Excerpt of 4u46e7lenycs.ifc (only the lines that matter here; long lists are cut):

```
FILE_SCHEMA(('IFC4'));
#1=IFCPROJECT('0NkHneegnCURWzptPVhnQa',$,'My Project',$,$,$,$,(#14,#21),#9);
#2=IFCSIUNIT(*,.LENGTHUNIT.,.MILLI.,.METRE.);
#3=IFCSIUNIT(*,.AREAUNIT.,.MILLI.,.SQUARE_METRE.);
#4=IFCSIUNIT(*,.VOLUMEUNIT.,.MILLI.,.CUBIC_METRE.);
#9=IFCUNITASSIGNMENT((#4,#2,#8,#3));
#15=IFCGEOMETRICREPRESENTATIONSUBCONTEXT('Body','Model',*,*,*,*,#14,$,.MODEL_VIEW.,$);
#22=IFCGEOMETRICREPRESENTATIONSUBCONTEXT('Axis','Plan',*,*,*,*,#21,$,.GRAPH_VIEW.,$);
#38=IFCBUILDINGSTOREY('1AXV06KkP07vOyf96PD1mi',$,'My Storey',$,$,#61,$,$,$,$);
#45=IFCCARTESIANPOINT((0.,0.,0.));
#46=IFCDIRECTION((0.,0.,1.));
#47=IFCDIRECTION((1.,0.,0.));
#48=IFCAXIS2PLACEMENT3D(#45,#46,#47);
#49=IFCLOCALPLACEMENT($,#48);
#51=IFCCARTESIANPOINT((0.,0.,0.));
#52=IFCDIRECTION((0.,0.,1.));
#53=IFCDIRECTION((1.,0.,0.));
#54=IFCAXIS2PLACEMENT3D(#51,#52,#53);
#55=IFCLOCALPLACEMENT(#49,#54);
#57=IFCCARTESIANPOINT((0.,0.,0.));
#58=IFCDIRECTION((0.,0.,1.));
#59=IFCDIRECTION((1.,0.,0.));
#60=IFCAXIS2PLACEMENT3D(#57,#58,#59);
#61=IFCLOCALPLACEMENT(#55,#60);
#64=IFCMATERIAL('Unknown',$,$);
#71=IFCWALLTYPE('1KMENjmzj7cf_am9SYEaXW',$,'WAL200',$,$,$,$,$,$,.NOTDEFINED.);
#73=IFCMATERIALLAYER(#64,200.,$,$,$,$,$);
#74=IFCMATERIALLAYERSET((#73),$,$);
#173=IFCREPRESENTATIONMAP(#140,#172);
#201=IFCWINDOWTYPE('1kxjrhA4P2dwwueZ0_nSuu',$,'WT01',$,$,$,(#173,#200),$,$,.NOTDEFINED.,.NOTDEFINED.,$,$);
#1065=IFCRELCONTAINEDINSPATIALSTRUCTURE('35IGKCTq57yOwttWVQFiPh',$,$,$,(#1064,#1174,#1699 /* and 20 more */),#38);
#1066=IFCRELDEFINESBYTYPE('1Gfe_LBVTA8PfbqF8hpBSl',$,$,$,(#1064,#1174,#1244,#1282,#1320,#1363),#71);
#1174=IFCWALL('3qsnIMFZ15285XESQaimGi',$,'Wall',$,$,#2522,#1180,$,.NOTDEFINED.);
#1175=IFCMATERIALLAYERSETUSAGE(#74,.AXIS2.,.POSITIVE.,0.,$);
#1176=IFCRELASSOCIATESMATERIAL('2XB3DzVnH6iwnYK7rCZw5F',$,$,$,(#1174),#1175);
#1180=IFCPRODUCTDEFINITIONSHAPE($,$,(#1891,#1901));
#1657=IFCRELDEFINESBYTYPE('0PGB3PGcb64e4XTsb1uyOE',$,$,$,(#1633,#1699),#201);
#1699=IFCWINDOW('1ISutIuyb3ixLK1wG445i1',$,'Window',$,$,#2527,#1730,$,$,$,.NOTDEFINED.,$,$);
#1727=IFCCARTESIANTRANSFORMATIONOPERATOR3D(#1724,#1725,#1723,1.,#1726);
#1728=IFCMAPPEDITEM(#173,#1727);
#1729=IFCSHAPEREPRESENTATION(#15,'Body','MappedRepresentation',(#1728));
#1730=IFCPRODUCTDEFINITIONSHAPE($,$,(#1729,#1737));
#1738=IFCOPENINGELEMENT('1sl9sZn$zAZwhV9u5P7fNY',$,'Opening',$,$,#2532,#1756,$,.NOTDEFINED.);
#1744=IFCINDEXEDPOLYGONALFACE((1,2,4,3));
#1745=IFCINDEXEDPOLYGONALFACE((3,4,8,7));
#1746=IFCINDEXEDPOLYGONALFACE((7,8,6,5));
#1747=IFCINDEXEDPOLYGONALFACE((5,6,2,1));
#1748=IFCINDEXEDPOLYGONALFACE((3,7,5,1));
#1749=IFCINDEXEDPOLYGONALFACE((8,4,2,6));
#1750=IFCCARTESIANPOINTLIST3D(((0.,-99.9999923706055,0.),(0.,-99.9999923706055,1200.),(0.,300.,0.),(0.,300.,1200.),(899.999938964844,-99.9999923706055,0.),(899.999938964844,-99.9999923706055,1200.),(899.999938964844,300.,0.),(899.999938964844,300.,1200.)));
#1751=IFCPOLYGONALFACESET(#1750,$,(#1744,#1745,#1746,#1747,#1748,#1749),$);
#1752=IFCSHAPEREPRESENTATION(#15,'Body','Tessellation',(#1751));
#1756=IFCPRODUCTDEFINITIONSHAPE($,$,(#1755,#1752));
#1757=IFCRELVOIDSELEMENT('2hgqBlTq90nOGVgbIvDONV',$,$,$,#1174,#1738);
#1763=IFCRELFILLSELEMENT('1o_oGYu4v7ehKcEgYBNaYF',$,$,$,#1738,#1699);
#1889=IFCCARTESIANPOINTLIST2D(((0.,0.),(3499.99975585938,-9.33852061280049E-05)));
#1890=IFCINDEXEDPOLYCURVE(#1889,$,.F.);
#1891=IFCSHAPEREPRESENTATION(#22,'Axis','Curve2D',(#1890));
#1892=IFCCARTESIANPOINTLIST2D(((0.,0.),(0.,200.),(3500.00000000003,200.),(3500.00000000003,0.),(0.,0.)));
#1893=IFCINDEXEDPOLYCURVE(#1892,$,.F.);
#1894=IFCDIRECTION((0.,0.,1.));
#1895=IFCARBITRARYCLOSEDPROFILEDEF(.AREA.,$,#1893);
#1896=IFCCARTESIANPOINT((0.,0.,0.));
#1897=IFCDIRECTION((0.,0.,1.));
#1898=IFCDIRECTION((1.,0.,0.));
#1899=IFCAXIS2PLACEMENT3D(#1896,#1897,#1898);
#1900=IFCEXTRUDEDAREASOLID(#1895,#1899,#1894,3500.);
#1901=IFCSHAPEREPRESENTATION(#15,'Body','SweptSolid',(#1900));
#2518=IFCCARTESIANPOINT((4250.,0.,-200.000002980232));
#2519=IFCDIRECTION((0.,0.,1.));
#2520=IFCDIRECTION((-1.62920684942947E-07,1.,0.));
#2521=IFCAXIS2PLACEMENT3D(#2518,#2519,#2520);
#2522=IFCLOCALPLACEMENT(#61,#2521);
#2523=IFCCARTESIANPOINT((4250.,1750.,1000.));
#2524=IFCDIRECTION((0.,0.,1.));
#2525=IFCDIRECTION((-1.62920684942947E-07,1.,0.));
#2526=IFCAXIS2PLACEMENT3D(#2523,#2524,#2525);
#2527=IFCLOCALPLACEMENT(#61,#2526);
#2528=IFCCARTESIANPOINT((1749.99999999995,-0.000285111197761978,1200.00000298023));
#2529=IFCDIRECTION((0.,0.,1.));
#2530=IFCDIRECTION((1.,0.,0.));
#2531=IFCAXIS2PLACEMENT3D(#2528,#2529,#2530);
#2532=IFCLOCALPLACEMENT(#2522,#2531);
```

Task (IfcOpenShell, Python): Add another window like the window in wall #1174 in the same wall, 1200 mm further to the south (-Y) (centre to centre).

```python
import ifcopenshell
import ifcopenshell.api.feature
import ifcopenshell.api.geometry
import ifcopenshell.api.root
import ifcopenshell.geom
import ifcopenshell.util.element
import ifcopenshell.util.placement
import ifcopenshell.util.shape
import ifcopenshell.util.unit

model = ifcopenshell.open("4u46e7lenycs.ifc")
unit_scale = ifcopenshell.util.unit.calculate_unit_scale(model)
settings = ifcopenshell.geom.settings()


def volume(element):
    """Net volume in cubic metres, openings subtracted."""
    shape = ifcopenshell.geom.create_shape(settings, element)
    return ifcopenshell.util.shape.get_volume(shape.geometry)


window = model.by_guid("1ISutIuyb3ixLK1wG445i1")
opening = window.FillsVoids[0].RelatingOpeningElement
wall = opening.VoidsElements[0].RelatingBuildingElement
before = volume(wall)
shift = ifcopenshell.util.placement.get_local_placement(wall.ObjectPlacement)[:3, 0] * -1.2 / unit_scale

# copy_class copies the void relationship, type, container and properties, but no geometry.
new_opening = ifcopenshell.api.root.copy_class(model, product=opening)
new_opening.Representation = ifcopenshell.util.element.copy_deep(
    model, opening.Representation, exclude=["IfcGeometricRepresentationContext", "IfcRepresentationMap"]
)
new_window = ifcopenshell.api.root.copy_class(model, product=window)
new_window.Representation = ifcopenshell.util.element.copy_deep(
    model, window.Representation, exclude=["IfcGeometricRepresentationContext", "IfcRepresentationMap"]
)
ifcopenshell.api.feature.add_filling(model, opening=new_opening, element=new_window)

for old, new in ((opening, new_opening), (window, new_window)):
    matrix = ifcopenshell.util.placement.get_local_placement(old.ObjectPlacement)
    matrix[:3, 3] += shift
    ifcopenshell.api.geometry.edit_object_placement(model, product=new, matrix=matrix, is_si=False)

after = volume(wall)

print(f"wall volume {before:.3f} -> {after:.3f} m3")

model.write("4u46e7lenycs_v2.ifc")
```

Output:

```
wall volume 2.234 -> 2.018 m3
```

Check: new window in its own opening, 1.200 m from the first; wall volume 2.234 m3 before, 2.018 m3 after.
